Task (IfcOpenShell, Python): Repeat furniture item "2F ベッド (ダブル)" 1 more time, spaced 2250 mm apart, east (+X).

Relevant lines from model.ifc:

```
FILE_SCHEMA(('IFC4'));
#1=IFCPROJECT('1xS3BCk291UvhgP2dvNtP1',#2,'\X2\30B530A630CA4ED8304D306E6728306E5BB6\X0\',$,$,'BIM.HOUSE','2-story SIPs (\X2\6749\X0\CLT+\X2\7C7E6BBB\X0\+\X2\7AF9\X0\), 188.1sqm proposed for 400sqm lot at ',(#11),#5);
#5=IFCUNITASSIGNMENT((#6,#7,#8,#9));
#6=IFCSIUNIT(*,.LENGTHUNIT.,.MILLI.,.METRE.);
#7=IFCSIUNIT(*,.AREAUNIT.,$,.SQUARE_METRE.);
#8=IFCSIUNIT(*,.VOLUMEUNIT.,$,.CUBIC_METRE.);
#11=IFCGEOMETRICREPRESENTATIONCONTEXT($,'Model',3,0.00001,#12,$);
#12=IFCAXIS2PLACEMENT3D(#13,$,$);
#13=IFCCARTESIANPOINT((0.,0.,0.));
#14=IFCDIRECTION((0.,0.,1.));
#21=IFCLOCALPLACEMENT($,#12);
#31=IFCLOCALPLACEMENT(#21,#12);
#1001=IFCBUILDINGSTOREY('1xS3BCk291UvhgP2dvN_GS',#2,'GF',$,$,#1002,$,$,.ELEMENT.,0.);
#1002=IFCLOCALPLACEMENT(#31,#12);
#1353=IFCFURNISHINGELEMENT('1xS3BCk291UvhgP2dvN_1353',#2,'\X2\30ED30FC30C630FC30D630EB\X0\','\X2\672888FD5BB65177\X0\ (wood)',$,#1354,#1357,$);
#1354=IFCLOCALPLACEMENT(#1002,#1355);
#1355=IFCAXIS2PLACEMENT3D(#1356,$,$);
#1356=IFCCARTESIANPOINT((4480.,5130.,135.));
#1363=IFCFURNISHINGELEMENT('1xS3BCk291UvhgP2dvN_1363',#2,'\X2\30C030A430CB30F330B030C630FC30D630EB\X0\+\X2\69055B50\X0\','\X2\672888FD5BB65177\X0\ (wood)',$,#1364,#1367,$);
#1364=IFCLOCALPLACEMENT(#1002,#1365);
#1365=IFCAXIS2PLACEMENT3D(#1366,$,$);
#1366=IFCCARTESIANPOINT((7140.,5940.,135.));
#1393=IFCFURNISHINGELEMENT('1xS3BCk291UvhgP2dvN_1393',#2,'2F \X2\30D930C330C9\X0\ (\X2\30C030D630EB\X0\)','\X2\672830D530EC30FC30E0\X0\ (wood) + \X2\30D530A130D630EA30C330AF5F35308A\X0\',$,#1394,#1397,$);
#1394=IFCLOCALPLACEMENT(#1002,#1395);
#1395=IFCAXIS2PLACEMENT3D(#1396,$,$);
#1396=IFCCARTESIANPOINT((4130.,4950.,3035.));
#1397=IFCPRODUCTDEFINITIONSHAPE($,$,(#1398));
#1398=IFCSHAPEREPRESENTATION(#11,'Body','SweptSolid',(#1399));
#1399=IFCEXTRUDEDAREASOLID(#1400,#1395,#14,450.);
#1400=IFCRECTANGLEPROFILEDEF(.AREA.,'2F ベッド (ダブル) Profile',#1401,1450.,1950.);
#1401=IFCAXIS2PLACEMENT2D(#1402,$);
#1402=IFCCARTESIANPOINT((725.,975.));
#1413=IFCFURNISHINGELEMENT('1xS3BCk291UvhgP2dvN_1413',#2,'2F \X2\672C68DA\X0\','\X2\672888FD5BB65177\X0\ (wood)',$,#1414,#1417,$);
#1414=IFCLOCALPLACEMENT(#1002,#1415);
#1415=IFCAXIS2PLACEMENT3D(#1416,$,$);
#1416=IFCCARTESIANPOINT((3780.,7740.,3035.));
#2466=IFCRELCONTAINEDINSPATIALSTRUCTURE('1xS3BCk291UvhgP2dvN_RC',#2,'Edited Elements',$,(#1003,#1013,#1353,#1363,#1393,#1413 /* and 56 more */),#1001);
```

```python
import numpy as np
import ifcopenshell
import ifcopenshell.api.geometry
import ifcopenshell.api.root
import ifcopenshell.util.element
import ifcopenshell.util.placement

model = ifcopenshell.open("model.ifc")


def reuse_history(source, copy):
    """copy_class also copies each property set's owner history, people and application; keep the originals."""
    for rel in copy.IsDefinedBy:
        if rel.is_a("IfcRelDefinesByProperties") and (history := rel.RelatingPropertyDefinition.OwnerHistory):
            rel.RelatingPropertyDefinition.OwnerHistory = source.OwnerHistory
            ifcopenshell.util.element.remove_deep2(model, history)


source = model.by_guid("1xS3BCk291UvhgP2dvN_1393")
base = ifcopenshell.util.placement.get_local_placement(source.ObjectPlacement)
step = np.array([1.0, 0.0, 0.0]) * 2250.0

for i in range(1, 2):
    copy = ifcopenshell.api.root.copy_class(model, product=source)
    copy.Representation = ifcopenshell.util.element.copy_deep(
        model, source.Representation, exclude=["IfcGeometricRepresentationContext", "IfcRepresentationMap"]
    )
    reuse_history(source, copy)
    matrix = base.copy()
    matrix[:3, 3] += i * step
    print("added at", matrix[:3, 3].round(3) + 0.0)
    ifcopenshell.api.geometry.edit_object_placement(model, product=copy, matrix=matrix, is_si=False)

model.write("model_rev.ifc")
```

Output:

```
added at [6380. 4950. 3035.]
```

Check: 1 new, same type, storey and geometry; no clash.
